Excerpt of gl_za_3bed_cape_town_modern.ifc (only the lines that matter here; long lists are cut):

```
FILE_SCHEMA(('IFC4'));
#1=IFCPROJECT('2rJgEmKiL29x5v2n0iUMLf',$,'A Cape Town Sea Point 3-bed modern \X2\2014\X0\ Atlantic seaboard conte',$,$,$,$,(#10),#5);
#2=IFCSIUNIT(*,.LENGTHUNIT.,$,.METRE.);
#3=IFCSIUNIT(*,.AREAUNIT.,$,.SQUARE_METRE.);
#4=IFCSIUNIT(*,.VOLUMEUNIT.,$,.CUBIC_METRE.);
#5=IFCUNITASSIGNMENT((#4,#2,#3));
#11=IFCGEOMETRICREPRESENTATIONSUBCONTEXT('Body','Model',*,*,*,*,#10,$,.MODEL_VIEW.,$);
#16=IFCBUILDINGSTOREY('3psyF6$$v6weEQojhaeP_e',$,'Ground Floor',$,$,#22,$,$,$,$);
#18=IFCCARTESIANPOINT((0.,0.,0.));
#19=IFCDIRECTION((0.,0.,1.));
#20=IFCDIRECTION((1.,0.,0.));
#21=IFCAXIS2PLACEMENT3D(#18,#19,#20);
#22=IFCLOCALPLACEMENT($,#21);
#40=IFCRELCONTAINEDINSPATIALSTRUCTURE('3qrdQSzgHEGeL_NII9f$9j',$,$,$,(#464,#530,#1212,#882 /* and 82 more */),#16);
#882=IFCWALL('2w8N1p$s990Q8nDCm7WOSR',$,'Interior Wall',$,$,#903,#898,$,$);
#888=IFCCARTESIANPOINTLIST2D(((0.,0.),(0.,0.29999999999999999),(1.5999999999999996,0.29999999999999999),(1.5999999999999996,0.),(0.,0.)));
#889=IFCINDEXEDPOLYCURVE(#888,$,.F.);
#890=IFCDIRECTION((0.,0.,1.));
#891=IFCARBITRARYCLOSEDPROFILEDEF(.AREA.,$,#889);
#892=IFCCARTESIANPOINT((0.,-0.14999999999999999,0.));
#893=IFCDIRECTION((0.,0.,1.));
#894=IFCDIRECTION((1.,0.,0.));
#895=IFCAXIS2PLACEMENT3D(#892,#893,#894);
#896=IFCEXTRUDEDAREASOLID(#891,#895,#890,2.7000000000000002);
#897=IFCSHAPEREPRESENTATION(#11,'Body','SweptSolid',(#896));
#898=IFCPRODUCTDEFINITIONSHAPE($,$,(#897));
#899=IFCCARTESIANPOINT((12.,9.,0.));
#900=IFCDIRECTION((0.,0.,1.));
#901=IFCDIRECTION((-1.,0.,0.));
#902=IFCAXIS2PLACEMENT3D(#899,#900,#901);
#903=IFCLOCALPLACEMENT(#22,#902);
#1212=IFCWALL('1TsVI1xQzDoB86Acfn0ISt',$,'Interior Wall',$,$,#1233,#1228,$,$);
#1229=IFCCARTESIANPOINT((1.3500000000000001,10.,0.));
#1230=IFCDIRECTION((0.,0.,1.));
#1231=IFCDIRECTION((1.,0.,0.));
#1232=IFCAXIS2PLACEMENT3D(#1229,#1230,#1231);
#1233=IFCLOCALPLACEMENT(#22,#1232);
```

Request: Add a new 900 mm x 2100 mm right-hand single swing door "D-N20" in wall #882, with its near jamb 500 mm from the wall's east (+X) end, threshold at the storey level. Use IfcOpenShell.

```python
import numpy as np
import ifcopenshell
import ifcopenshell.api.feature
import ifcopenshell.api.geometry
import ifcopenshell.api.root
import ifcopenshell.api.spatial
import ifcopenshell.geom
import ifcopenshell.util.element
import ifcopenshell.util.placement
import ifcopenshell.util.representation
import ifcopenshell.util.shape
import ifcopenshell.util.unit

model = ifcopenshell.open("gl_za_3bed_cape_town_modern.ifc")
unit_scale = ifcopenshell.util.unit.calculate_unit_scale(model)
settings = ifcopenshell.geom.settings()


def volume(element):
    """Net volume in cubic metres, openings subtracted."""
    shape = ifcopenshell.geom.create_shape(settings, element)
    return ifcopenshell.util.shape.get_volume(shape.geometry)


wall = model.by_guid("2w8N1p$s990Q8nDCm7WOSR")
storey = ifcopenshell.util.element.get_container(wall, ifc_class="IfcBuildingStorey")
context = ifcopenshell.util.representation.get_context(model, "Model", "Body", "MODEL_VIEW")
before = volume(wall)

width, height, from_end, sill = 0.9, 2.1, 0.5, 0.0  # metres

# The wall runs along its own X axis, and the end named is its -X end.
wall_shape = ifcopenshell.geom.create_shape(settings, wall)
x, y, z = ifcopenshell.util.shape.get_vertices(wall_shape.geometry).T
start = x.min() + from_end
face, thickness = float(y.min()), float(y.max() - y.min())
wall_matrix = ifcopenshell.util.placement.get_local_placement(wall.ObjectPlacement)
level = ifcopenshell.util.placement.get_local_placement(storey.ObjectPlacement)[2, 3]


def in_wall(x, y):
    """Placement at x, y metres in the wall's axes, at sill height."""
    matrix = wall_matrix.copy()
    matrix[:, 3] = wall_matrix @ np.array([x / unit_scale, y / unit_scale, 0.0, 1.0])
    matrix[2, 3] = level + sill / unit_scale
    return matrix


# Opening: a box that overshoots both wall faces by 50 mm.
opening = ifcopenshell.api.root.create_entity(model, ifc_class="IfcOpeningElement", predefined_type="OPENING")
box = ifcopenshell.api.geometry.add_wall_representation(
    model, context=context, length=width, height=height, thickness=thickness + 0.1
)
ifcopenshell.api.geometry.assign_representation(model, product=opening, representation=box)
ifcopenshell.api.geometry.edit_object_placement(model, product=opening, matrix=in_wall(start, face - 0.05), is_si=False)
ifcopenshell.api.feature.add_feature(model, feature=opening, element=wall)

door = ifcopenshell.api.root.create_entity(model, ifc_class="IfcDoor", name="D-N20", predefined_type="DOOR")
door.OverallWidth, door.OverallHeight = width / unit_scale, height / unit_scale
door.OperationType = "SINGLE_SWING_RIGHT"
body = ifcopenshell.api.geometry.add_door_representation(
    model,
    context=context,
    overall_width=door.OverallWidth,
    overall_height=door.OverallHeight,
    operation_type="SINGLE_SWING_RIGHT",
    lining_properties={"LiningDepth": thickness / unit_scale, "ThresholdDepth": thickness / unit_scale},
)
ifcopenshell.api.geometry.assign_representation(model, product=door, representation=body)
ifcopenshell.api.spatial.assign_container(model, products=[door], relating_structure=storey)
ifcopenshell.api.feature.add_filling(model, opening=opening, element=door)

# The lining spans the wall, so the door starts at the wall face.
ifcopenshell.api.geometry.edit_object_placement(model, product=door, matrix=in_wall(start, face), is_si=False)

after = volume(wall)

print(f"wall volume {before:.3f} -> {after:.3f} m3")

model.write("gl_za_3bed_cape_town_modern-out.ifc")
```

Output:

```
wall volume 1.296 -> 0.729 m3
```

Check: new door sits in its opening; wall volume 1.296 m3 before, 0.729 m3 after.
